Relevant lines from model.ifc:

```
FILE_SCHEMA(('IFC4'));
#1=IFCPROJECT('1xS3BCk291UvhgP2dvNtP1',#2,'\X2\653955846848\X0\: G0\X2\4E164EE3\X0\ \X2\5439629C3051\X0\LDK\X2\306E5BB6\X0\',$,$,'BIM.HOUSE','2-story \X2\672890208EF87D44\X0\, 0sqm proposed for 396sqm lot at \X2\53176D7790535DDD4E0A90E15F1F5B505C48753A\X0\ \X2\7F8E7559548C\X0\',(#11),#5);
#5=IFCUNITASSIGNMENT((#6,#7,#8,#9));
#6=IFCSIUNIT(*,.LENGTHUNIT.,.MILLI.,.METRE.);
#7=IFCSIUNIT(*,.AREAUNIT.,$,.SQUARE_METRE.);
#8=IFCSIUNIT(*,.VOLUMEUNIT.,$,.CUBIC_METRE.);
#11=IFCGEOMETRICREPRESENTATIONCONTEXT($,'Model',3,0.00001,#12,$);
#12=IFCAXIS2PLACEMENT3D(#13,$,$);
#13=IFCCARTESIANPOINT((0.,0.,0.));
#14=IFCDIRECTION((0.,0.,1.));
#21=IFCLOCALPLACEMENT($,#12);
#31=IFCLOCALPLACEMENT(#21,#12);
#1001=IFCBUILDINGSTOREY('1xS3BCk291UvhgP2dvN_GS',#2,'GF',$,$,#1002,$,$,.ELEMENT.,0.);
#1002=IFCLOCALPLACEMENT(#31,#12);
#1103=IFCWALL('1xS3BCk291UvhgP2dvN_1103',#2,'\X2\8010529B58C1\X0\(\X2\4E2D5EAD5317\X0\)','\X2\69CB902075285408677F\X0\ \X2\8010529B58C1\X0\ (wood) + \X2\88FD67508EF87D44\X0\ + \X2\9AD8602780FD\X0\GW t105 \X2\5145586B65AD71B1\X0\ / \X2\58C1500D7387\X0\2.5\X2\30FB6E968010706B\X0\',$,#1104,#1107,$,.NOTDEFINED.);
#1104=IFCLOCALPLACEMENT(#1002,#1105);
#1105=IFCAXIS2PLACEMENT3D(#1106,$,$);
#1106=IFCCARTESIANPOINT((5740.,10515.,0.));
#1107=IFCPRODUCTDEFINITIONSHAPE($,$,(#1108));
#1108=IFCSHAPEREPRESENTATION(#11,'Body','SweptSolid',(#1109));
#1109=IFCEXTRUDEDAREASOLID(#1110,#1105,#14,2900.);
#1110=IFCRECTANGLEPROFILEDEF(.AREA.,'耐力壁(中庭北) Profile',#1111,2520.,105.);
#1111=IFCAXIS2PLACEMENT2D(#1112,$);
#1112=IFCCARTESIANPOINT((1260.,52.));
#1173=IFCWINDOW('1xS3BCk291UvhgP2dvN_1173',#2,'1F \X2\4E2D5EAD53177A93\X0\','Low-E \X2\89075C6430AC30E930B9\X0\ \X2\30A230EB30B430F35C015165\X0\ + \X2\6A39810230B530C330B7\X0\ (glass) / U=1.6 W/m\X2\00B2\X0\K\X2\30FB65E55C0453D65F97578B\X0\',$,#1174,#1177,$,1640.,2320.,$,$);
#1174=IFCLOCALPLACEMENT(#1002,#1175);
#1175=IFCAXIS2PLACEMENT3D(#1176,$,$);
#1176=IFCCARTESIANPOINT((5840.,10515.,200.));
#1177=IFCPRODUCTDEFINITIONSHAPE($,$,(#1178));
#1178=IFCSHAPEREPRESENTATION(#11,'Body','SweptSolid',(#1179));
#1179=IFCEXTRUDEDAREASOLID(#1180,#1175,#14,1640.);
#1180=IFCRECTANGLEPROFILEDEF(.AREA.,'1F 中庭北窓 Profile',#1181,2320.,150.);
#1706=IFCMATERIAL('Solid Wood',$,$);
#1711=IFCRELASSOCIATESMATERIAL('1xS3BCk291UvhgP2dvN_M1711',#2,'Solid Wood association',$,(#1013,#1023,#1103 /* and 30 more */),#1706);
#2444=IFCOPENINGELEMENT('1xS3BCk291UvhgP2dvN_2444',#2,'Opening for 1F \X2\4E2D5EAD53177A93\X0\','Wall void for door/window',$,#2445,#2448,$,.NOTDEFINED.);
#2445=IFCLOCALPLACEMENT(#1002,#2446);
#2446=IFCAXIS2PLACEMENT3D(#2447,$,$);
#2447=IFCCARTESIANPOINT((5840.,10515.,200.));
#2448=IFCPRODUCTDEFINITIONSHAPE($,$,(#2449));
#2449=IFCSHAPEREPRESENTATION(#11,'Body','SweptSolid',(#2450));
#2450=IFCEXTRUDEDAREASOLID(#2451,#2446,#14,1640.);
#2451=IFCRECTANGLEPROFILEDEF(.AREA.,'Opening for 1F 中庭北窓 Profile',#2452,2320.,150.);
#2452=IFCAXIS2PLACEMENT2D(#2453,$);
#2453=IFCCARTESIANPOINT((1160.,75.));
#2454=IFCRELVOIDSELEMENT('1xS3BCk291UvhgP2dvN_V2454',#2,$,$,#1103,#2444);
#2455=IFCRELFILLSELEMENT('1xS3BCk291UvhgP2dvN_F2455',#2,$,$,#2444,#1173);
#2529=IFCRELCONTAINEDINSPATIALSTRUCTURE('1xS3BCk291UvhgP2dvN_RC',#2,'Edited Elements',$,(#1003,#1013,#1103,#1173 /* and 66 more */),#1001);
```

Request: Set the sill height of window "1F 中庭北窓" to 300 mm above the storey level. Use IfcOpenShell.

```python
import numpy as np
import ifcopenshell
import ifcopenshell.api.geometry
import ifcopenshell.geom
import ifcopenshell.util.element
import ifcopenshell.util.placement
import ifcopenshell.util.shape
import ifcopenshell.util.unit

model = ifcopenshell.open("model.ifc")
unit_scale = ifcopenshell.util.unit.calculate_unit_scale(model)

window = model.by_guid("1xS3BCk291UvhgP2dvN_1173")
opening = window.FillsVoids[0].RelatingOpeningElement
storey = ifcopenshell.util.element.get_container(window, ifc_class="IfcBuildingStorey")
level = ifcopenshell.util.placement.get_local_placement(storey.ObjectPlacement)[2, 3]

# The opening's origin need not be at the sill, so measure its lowest point.
shape = ifcopenshell.geom.create_shape(ifcopenshell.geom.settings(), opening)
bottom = ifcopenshell.util.shape.get_shape_bottom_elevation(shape, shape.geometry) / unit_scale
dz = level + 0.3 / unit_scale - bottom

shift = np.array([0.0, 0.0, dz])
# The window is not placed relative to its opening, so move both.
for product in (opening, window):
    matrix = ifcopenshell.util.placement.get_local_placement(product.ObjectPlacement)
    matrix[:3, 3] += shift
    ifcopenshell.api.geometry.edit_object_placement(model, product=product, matrix=matrix, is_si=False)

print(f"moved by {dz * unit_scale:+.3f} m")

model.write("model-out.ifc")
```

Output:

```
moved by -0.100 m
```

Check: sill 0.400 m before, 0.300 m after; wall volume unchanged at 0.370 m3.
